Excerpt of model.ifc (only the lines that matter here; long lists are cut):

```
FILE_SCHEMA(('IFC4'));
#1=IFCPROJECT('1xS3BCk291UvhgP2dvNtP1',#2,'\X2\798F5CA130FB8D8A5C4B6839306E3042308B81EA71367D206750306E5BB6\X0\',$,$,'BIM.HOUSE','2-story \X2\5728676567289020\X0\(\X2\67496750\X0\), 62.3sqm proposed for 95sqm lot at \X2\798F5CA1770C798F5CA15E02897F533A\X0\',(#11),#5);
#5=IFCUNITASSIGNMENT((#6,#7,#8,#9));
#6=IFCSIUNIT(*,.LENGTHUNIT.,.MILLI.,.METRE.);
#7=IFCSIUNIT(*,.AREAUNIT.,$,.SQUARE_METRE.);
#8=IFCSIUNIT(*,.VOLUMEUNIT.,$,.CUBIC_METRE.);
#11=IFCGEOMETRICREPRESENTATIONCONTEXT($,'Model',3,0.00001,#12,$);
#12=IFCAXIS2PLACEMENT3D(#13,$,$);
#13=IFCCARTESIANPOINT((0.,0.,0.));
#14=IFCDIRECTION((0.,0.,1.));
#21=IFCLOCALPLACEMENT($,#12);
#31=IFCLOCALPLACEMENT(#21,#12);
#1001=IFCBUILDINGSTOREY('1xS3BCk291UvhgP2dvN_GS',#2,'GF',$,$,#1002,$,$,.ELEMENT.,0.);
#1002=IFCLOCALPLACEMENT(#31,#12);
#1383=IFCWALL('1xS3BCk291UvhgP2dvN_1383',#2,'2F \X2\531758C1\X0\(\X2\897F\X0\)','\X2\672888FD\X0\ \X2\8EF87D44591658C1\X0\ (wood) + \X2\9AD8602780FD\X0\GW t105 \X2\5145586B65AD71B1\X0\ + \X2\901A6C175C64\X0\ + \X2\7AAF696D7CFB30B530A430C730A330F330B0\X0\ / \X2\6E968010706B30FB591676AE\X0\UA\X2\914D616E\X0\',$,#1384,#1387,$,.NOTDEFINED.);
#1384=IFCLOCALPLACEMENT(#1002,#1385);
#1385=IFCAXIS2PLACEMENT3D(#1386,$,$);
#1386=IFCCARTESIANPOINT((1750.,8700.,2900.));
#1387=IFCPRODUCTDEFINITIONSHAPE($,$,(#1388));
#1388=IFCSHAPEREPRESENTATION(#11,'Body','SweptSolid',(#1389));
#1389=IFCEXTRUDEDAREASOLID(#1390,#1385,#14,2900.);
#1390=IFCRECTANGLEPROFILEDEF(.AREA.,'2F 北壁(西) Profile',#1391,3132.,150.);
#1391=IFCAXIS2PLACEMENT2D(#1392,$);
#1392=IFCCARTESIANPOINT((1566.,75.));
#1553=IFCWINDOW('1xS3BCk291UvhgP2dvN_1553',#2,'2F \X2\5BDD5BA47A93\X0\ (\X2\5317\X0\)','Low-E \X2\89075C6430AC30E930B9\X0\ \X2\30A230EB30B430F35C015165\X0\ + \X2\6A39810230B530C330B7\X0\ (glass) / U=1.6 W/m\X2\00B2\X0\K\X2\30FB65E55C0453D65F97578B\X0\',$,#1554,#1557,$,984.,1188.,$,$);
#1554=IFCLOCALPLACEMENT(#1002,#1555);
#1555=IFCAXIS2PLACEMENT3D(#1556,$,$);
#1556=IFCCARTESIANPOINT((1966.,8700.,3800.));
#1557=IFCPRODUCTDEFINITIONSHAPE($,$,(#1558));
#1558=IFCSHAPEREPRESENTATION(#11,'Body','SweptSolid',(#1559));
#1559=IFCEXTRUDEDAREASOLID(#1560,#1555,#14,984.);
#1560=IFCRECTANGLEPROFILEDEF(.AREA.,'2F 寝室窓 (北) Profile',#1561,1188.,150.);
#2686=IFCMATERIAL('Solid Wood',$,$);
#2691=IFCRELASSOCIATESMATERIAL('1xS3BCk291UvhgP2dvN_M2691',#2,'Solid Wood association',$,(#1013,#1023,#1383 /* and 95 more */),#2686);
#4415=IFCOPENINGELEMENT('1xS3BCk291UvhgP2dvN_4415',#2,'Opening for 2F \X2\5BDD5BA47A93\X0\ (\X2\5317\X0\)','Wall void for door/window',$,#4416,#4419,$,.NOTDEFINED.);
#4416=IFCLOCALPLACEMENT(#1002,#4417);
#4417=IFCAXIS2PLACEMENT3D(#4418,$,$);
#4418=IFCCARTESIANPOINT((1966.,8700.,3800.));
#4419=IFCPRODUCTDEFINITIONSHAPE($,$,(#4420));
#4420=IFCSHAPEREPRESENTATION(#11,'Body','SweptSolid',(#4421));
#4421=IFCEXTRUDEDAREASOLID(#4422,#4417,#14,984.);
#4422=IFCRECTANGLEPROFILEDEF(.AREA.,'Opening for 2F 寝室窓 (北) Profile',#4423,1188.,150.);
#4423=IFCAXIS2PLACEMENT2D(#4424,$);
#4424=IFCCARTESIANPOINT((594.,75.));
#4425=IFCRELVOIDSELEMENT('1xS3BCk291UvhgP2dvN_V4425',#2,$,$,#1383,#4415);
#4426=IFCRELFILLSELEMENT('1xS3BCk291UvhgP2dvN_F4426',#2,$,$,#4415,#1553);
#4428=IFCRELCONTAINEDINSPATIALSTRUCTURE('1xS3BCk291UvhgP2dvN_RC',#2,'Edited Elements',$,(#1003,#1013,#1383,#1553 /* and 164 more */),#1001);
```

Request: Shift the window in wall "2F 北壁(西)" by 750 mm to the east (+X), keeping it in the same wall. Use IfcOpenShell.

```python
import ifcopenshell
import ifcopenshell.api.geometry
import ifcopenshell.util.placement
import ifcopenshell.util.unit

model = ifcopenshell.open("model.ifc")
unit_scale = ifcopenshell.util.unit.calculate_unit_scale(model)

window = model.by_guid("1xS3BCk291UvhgP2dvN_1553")
opening = window.FillsVoids[0].RelatingOpeningElement
wall = opening.VoidsElements[0].RelatingBuildingElement

wall_matrix = ifcopenshell.util.placement.get_local_placement(wall.ObjectPlacement)
shift = wall_matrix[:3, 0] * 0.75 / unit_scale
before = ifcopenshell.util.placement.get_local_placement(window.ObjectPlacement)[:3, 3].copy()

# The window is not placed relative to its opening, so move both.
for product in (opening, window):
    matrix = ifcopenshell.util.placement.get_local_placement(product.ObjectPlacement)
    matrix[:3, 3] += shift
    ifcopenshell.api.geometry.edit_object_placement(model, product=product, matrix=matrix, is_si=False)

after = ifcopenshell.util.placement.get_local_placement(window.ObjectPlacement)[:3, 3]
print("window moved by", (after - before).round(3) + 0.0)

model.write("model_rev.ifc")
```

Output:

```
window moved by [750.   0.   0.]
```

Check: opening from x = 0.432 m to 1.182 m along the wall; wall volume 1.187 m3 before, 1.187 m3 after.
